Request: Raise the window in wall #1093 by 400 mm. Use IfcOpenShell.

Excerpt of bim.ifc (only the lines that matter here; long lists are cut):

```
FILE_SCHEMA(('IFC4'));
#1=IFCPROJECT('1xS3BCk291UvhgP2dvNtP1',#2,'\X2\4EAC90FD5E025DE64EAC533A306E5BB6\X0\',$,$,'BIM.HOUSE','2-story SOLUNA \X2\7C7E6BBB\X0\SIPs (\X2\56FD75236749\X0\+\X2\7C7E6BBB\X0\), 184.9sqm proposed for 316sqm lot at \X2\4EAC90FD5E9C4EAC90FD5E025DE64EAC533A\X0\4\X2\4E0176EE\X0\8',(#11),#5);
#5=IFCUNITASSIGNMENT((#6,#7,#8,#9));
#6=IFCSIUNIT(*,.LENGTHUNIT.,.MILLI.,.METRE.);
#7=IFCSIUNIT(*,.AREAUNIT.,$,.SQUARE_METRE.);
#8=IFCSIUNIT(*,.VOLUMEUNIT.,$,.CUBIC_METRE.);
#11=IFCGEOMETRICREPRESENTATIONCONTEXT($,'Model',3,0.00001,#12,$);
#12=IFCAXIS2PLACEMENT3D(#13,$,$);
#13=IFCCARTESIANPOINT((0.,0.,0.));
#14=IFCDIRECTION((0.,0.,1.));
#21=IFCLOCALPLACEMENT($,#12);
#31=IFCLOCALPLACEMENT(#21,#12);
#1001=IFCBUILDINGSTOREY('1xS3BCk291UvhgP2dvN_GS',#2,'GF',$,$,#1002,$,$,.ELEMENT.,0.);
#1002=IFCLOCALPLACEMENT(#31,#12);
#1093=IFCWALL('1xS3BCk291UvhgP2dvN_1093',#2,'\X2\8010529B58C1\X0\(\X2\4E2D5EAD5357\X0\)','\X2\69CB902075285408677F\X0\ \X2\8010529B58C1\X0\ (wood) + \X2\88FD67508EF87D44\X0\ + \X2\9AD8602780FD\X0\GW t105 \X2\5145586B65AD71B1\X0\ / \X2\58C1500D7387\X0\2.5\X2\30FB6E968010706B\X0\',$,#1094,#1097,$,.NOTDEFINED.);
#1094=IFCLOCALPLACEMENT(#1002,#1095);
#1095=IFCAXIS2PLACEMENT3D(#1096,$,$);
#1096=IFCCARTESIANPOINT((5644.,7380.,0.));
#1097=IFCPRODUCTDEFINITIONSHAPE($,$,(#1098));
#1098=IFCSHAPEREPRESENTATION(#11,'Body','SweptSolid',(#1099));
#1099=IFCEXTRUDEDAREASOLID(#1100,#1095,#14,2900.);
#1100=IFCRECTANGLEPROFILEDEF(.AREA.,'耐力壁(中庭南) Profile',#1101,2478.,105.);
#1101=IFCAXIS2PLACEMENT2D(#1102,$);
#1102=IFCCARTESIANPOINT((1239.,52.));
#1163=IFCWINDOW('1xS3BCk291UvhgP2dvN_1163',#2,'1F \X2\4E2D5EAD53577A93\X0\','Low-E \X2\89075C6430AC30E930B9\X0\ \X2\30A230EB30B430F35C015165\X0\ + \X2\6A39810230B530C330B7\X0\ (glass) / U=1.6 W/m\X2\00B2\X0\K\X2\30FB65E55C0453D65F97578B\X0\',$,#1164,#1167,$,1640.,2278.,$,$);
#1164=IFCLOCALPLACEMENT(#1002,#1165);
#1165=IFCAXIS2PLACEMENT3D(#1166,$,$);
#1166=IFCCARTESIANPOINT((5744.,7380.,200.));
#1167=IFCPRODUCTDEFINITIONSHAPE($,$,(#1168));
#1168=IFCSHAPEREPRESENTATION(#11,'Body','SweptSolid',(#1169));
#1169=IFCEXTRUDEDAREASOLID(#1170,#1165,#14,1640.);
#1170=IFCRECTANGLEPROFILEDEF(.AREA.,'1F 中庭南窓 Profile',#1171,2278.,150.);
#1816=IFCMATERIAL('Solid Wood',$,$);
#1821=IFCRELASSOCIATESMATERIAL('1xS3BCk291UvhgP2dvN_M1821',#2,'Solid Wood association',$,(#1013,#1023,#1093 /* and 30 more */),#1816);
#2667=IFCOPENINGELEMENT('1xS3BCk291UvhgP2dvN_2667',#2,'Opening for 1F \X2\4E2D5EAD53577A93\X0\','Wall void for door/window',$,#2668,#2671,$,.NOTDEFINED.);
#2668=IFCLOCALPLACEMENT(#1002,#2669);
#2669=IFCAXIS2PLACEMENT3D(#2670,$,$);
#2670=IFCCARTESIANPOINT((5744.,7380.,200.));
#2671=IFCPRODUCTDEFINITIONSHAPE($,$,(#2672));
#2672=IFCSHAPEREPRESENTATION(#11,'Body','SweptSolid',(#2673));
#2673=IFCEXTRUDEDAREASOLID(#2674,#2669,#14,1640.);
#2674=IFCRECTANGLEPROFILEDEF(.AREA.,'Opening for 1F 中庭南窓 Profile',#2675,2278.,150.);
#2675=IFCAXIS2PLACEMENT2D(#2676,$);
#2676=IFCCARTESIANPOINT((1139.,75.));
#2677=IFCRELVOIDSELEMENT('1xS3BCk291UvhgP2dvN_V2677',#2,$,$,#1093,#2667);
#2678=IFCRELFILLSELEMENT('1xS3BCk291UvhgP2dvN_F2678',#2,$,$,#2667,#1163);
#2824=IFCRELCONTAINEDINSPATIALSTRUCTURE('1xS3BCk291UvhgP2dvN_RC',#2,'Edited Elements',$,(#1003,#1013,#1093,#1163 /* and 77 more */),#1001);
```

```python
import numpy as np
import ifcopenshell
import ifcopenshell.api.geometry
import ifcopenshell.util.placement
import ifcopenshell.util.unit

model = ifcopenshell.open("bim.ifc")
unit_scale = ifcopenshell.util.unit.calculate_unit_scale(model)

window = model.by_guid("1xS3BCk291UvhgP2dvN_1163")
opening = window.FillsVoids[0].RelatingOpeningElement
dz = 0.4 / unit_scale

shift = np.array([0.0, 0.0, dz])
# The window is not placed relative to its opening, so move both.
for product in (opening, window):
    matrix = ifcopenshell.util.placement.get_local_placement(product.ObjectPlacement)
    matrix[:3, 3] += shift
    ifcopenshell.api.geometry.edit_object_placement(model, product=product, matrix=matrix, is_si=False)

print(f"moved by {dz * unit_scale:+.3f} m")

model.write("bim_edited.ifc")
```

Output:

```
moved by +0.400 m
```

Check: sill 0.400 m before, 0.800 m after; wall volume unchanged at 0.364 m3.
